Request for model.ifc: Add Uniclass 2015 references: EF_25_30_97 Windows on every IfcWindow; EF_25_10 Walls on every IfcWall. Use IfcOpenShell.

First a look at what the model holds.

```python
import ifcopenshell

model = ifcopenshell.open("model.ifc")
print(model.schema)
print("classifications:", [c.Name for c in model.by_type("IfcClassification")])
for ifc_class in ("IfcDoor", "IfcRoof", "IfcStair", "IfcWall", "IfcWindow"):
    print(ifc_class, len(model.by_type(ifc_class)))
```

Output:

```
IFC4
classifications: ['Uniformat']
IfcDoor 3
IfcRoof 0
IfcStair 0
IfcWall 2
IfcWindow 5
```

```python
import ifcopenshell
import ifcopenshell.api.classification

model = ifcopenshell.open("model.ifc")

system = ifcopenshell.api.classification.add_classification(model, classification="Uniclass 2015")

codes = {
    "IfcWindow": ("EF_25_30_97", "Windows"),
    "IfcWall": ("EF_25_10", "Walls"),
}
for ifc_class, (code, name) in codes.items():
    products = model.by_type(ifc_class)
    ifcopenshell.api.classification.add_reference(
        model, products=products, classification=system, identification=code, name=name
    )
    print(code, len(products))

model.write("model_rev.ifc")
```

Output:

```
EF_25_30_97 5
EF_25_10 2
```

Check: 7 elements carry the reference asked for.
